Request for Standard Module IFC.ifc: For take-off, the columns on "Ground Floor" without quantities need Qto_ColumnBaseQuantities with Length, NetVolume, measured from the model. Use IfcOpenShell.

First a look at what the model holds.

```python
import ifcopenshell
import ifcopenshell.util.element
import ifcopenshell.util.unit

model = ifcopenshell.open("Standard Module IFC.ifc")
print(model.schema)
for unit_type in ("LENGTHUNIT", "AREAUNIT", "VOLUMEUNIT"):
    print(unit_type, ifcopenshell.util.unit.calculate_unit_scale(model, unit_type))
storey = next(s for s in model.by_type("IfcBuildingStorey") if s.Name == "Ground Floor")
columns = [e for e in ifcopenshell.util.element.get_decomposition(storey) if e.is_a("IfcColumn")]
for e in sorted(columns, key=lambda e: e.id()):
    print(e.id(), e.is_a(), e.Name, list(ifcopenshell.util.element.get_psets(e, qtos_only=True)), sep=" | ")
```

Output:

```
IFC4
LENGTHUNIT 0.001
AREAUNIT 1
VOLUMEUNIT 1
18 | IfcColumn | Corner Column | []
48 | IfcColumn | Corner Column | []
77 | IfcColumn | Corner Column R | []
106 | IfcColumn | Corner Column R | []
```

```python
import ifcopenshell
import ifcopenshell.api.pset
import ifcopenshell.geom
import ifcopenshell.util.element
import ifcopenshell.util.shape
import ifcopenshell.util.unit

model = ifcopenshell.open("Standard Module IFC.ifc")
unit_scale = ifcopenshell.util.unit.calculate_unit_scale(model)
volume_scale = ifcopenshell.util.unit.calculate_unit_scale(model, "VOLUMEUNIT")
settings = ifcopenshell.geom.settings()

storey = next(s for s in model.by_type("IfcBuildingStorey") if s.Name == "Ground Floor")
columns = [e for e in ifcopenshell.util.element.get_decomposition(storey) if e.is_a("IfcColumn")]

for e in sorted(columns, key=lambda e: e.id()):
    if ifcopenshell.util.element.get_psets(e, qtos_only=True, should_inherit=False):
        continue
    # Geometry comes back in metres, in the element's own axes.
    shape = ifcopenshell.geom.create_shape(settings, e)
    values = {
        "Length": ifcopenshell.util.shape.get_z(shape.geometry) / unit_scale,
        "NetVolume": ifcopenshell.util.shape.get_volume(shape.geometry) / volume_scale,
    }
    qto = ifcopenshell.api.pset.add_qto(model, product=e, name="Qto_ColumnBaseQuantities")
    ifcopenshell.api.pset.edit_qto(model, qto=qto, properties=values)
    print(e.id(), {k: round(v, 3) for k, v in values.items()})

model.write("Standard Module IFC_v2.ifc")
```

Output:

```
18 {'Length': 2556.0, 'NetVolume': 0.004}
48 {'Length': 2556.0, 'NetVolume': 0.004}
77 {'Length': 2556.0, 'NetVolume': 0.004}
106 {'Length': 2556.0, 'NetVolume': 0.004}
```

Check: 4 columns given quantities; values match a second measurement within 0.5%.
